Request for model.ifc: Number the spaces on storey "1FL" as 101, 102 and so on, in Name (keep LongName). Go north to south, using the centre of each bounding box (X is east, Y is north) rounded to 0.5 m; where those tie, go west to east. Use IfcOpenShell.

First a look at what the model holds.

```python
import ifcopenshell
import ifcopenshell.util.element
import ifcopenshell.util.placement

model = ifcopenshell.open("model.ifc")
print(model.schema)
storey = next(s for s in model.by_type("IfcBuildingStorey") if s.Name == "1FL")
spaces = [e for e in ifcopenshell.util.element.get_decomposition(storey) if e.is_a("IfcSpace")]
for e in sorted(spaces, key=lambda e: e.id()):
    origin = ifcopenshell.util.placement.get_local_placement(e.ObjectPlacement)[:3, 3]
    print(e.id(), e.Name, e.LongName, origin.round(2) + 0.0, sep=" | ")
```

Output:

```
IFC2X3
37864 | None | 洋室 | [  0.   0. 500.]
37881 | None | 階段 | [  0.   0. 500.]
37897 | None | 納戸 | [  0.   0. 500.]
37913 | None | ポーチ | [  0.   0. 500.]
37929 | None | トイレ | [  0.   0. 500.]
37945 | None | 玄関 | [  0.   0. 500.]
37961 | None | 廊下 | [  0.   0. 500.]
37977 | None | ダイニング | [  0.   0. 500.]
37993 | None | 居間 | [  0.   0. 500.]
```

```python
import ifcopenshell
import ifcopenshell.geom
import ifcopenshell.util.element
import ifcopenshell.util.shape

model = ifcopenshell.open("model.ifc")
settings = ifcopenshell.geom.settings()
settings.set("use-world-coords", True)


def centre(element):
    shape = ifcopenshell.geom.create_shape(settings, element)
    return ifcopenshell.util.shape.get_bbox_centroid(shape.geometry)


storey = next(s for s in model.by_type("IfcBuildingStorey") if s.Name == "1FL")
spaces = [e for e in ifcopenshell.util.element.get_decomposition(storey) if e.is_a("IfcSpace")]

# Insertion points can sit at a corner or the storey origin, so sort by the geometry (in metres).
centres = {e: centre(e) for e in spaces}
spaces.sort(key=lambda e: (-round(centres[e][1] / 0.5), centres[e][0]))

for i, e in enumerate(spaces, start=1):
    number = f"1{i:02d}"
    e.Name = number
    print(e.id(), number)

model.write("model_edited.ifc")
```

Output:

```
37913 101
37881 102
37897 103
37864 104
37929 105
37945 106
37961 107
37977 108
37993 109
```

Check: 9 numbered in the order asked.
